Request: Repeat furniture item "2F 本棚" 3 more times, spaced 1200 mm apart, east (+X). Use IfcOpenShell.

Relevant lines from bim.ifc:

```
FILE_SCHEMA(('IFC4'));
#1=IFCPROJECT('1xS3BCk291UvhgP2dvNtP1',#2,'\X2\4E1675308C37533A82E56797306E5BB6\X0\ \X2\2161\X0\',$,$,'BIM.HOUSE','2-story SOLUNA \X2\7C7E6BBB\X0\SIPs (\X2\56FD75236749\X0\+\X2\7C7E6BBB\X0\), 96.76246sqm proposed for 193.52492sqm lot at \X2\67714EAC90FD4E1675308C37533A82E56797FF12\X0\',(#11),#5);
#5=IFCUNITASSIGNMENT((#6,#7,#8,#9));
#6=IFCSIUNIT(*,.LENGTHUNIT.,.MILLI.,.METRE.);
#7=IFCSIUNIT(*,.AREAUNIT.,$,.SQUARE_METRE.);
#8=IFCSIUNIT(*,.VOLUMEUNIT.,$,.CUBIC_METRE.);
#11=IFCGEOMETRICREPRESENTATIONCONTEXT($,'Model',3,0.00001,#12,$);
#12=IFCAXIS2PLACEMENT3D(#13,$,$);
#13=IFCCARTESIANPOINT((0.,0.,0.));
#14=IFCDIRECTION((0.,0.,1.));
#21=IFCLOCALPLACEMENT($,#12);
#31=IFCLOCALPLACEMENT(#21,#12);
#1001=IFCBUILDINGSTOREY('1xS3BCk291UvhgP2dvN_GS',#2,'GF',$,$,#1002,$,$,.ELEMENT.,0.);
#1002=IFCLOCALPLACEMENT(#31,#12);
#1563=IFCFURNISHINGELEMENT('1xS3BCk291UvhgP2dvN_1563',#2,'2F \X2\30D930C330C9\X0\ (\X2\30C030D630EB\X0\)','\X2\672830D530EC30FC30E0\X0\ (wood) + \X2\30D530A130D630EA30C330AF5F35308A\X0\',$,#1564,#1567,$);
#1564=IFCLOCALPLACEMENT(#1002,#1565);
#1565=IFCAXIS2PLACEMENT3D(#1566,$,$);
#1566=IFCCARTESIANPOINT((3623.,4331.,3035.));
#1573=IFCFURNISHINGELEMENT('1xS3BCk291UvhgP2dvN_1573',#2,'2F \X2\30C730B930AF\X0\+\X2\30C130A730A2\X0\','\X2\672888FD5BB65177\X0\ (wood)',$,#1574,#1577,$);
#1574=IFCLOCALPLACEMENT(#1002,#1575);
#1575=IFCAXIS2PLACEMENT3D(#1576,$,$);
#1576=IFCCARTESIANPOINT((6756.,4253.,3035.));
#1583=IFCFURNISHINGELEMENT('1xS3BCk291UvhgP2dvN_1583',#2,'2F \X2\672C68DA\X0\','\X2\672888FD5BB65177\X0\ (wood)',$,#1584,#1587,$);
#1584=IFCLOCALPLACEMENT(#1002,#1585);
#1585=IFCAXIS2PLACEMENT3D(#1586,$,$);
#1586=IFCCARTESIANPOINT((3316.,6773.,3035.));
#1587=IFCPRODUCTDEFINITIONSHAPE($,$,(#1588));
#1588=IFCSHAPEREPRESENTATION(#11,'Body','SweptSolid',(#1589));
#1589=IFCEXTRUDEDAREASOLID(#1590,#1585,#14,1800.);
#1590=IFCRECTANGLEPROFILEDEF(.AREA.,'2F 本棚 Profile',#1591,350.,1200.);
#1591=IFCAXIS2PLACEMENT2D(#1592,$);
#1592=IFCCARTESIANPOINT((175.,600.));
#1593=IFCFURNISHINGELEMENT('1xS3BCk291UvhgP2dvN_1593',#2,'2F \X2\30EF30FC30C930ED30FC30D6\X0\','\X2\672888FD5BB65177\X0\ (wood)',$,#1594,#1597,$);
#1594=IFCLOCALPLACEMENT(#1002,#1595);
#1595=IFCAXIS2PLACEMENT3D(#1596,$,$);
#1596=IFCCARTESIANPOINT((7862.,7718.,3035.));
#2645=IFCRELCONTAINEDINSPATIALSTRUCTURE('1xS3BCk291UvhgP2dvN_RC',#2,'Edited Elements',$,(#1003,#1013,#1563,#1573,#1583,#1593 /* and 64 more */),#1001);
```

```python
import numpy as np
import ifcopenshell
import ifcopenshell.api.geometry
import ifcopenshell.api.root
import ifcopenshell.util.element
import ifcopenshell.util.placement
import ifcopenshell.util.unit

model = ifcopenshell.open("bim.ifc")
unit_scale = ifcopenshell.util.unit.calculate_unit_scale(model)


def reuse_history(source, copy):
    """copy_class also copies each property set's owner history, people and application; keep the originals."""
    for rel in copy.IsDefinedBy:
        if rel.is_a("IfcRelDefinesByProperties") and (history := rel.RelatingPropertyDefinition.OwnerHistory):
            rel.RelatingPropertyDefinition.OwnerHistory = source.OwnerHistory
            ifcopenshell.util.element.remove_deep2(model, history)


source = model.by_guid("1xS3BCk291UvhgP2dvN_1583")
base = ifcopenshell.util.placement.get_local_placement(source.ObjectPlacement)
step = np.array([1.0, 0.0, 0.0]) * 1.2 / unit_scale

for i in range(1, 4):
    copy = ifcopenshell.api.root.copy_class(model, product=source)
    copy.Representation = ifcopenshell.util.element.copy_deep(
        model, source.Representation, exclude=["IfcGeometricRepresentationContext", "IfcRepresentationMap"]
    )
    reuse_history(source, copy)
    matrix = base.copy()
    matrix[:3, 3] += i * step
    print("added at", matrix[:3, 3].round(3) + 0.0)
    ifcopenshell.api.geometry.edit_object_placement(model, product=copy, matrix=matrix, is_si=False)

model.write("bim_updated.ifc")
```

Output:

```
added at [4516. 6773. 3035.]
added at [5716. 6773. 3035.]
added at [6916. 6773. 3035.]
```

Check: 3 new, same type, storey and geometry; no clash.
